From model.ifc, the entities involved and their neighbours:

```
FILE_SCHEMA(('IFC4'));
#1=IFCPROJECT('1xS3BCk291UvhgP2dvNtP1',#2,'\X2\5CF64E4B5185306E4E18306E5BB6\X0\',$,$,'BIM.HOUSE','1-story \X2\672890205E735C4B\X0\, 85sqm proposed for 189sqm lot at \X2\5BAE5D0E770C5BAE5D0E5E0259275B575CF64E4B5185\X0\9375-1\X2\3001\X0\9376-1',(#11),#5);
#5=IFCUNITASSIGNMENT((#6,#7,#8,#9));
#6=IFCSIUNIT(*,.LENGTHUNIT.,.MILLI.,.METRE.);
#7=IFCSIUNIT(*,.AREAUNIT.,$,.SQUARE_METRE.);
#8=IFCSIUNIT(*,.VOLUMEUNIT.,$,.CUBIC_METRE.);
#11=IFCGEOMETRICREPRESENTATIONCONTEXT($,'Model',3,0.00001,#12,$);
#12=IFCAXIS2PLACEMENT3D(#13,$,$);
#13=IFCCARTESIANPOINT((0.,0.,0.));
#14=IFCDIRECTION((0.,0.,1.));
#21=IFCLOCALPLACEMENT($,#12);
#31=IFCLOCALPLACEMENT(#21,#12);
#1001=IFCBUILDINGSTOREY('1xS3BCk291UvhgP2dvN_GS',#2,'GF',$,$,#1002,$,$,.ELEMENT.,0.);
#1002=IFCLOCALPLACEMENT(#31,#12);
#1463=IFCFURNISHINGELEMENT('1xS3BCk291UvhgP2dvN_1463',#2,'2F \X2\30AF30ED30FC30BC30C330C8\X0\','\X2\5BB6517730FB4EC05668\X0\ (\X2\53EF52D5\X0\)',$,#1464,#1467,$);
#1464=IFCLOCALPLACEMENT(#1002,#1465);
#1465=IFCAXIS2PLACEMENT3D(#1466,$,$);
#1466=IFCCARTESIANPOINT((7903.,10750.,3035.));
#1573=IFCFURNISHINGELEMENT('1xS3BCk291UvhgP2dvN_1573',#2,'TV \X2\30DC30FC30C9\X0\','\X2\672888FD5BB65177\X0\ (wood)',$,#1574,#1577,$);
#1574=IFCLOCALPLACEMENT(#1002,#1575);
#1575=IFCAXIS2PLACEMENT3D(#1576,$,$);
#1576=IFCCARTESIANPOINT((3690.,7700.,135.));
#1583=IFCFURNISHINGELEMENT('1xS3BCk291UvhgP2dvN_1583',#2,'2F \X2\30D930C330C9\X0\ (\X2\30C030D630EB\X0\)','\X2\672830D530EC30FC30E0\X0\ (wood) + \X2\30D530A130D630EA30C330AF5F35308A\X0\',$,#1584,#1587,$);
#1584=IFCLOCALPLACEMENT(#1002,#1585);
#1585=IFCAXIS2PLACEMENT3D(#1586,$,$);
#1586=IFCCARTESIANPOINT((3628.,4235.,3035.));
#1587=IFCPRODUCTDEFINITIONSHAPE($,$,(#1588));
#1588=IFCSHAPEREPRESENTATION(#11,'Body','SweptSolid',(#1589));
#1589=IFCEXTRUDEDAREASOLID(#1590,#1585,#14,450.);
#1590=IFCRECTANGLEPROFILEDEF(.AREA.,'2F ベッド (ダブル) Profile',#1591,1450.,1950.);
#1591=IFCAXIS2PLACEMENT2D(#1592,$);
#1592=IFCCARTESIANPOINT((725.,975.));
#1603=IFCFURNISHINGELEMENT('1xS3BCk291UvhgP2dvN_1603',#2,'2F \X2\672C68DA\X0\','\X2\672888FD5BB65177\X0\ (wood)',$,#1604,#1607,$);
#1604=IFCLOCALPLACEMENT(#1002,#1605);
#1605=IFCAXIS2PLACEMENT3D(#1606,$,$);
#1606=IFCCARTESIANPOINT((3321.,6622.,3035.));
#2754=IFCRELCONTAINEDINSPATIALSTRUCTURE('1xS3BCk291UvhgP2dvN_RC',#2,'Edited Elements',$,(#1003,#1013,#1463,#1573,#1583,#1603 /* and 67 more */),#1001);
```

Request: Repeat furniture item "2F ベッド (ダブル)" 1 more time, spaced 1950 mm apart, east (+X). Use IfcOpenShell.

```python
import numpy as np
import ifcopenshell
import ifcopenshell.api.geometry
import ifcopenshell.api.root
import ifcopenshell.util.element
import ifcopenshell.util.placement
import ifcopenshell.util.unit

model = ifcopenshell.open("model.ifc")
unit_scale = ifcopenshell.util.unit.calculate_unit_scale(model)


def reuse_history(source, copy):
    """copy_class also copies each property set's owner history, people and application; keep the originals."""
    for rel in copy.IsDefinedBy:
        if rel.is_a("IfcRelDefinesByProperties") and (history := rel.RelatingPropertyDefinition.OwnerHistory):
            rel.RelatingPropertyDefinition.OwnerHistory = source.OwnerHistory
            ifcopenshell.util.element.remove_deep2(model, history)


source = model.by_guid("1xS3BCk291UvhgP2dvN_1583")
base = ifcopenshell.util.placement.get_local_placement(source.ObjectPlacement)
step = np.array([1.0, 0.0, 0.0]) * 1.95 / unit_scale

for i in range(1, 2):
    copy = ifcopenshell.api.root.copy_class(model, product=source)
    copy.Representation = ifcopenshell.util.element.copy_deep(
        model, source.Representation, exclude=["IfcGeometricRepresentationContext", "IfcRepresentationMap"]
    )
    reuse_history(source, copy)
    matrix = base.copy()
    matrix[:3, 3] += i * step
    print("added at", matrix[:3, 3].round(3) + 0.0)
    ifcopenshell.api.geometry.edit_object_placement(model, product=copy, matrix=matrix, is_si=False)

model.write("model_edited.ifc")
```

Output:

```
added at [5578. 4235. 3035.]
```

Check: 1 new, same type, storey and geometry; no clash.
